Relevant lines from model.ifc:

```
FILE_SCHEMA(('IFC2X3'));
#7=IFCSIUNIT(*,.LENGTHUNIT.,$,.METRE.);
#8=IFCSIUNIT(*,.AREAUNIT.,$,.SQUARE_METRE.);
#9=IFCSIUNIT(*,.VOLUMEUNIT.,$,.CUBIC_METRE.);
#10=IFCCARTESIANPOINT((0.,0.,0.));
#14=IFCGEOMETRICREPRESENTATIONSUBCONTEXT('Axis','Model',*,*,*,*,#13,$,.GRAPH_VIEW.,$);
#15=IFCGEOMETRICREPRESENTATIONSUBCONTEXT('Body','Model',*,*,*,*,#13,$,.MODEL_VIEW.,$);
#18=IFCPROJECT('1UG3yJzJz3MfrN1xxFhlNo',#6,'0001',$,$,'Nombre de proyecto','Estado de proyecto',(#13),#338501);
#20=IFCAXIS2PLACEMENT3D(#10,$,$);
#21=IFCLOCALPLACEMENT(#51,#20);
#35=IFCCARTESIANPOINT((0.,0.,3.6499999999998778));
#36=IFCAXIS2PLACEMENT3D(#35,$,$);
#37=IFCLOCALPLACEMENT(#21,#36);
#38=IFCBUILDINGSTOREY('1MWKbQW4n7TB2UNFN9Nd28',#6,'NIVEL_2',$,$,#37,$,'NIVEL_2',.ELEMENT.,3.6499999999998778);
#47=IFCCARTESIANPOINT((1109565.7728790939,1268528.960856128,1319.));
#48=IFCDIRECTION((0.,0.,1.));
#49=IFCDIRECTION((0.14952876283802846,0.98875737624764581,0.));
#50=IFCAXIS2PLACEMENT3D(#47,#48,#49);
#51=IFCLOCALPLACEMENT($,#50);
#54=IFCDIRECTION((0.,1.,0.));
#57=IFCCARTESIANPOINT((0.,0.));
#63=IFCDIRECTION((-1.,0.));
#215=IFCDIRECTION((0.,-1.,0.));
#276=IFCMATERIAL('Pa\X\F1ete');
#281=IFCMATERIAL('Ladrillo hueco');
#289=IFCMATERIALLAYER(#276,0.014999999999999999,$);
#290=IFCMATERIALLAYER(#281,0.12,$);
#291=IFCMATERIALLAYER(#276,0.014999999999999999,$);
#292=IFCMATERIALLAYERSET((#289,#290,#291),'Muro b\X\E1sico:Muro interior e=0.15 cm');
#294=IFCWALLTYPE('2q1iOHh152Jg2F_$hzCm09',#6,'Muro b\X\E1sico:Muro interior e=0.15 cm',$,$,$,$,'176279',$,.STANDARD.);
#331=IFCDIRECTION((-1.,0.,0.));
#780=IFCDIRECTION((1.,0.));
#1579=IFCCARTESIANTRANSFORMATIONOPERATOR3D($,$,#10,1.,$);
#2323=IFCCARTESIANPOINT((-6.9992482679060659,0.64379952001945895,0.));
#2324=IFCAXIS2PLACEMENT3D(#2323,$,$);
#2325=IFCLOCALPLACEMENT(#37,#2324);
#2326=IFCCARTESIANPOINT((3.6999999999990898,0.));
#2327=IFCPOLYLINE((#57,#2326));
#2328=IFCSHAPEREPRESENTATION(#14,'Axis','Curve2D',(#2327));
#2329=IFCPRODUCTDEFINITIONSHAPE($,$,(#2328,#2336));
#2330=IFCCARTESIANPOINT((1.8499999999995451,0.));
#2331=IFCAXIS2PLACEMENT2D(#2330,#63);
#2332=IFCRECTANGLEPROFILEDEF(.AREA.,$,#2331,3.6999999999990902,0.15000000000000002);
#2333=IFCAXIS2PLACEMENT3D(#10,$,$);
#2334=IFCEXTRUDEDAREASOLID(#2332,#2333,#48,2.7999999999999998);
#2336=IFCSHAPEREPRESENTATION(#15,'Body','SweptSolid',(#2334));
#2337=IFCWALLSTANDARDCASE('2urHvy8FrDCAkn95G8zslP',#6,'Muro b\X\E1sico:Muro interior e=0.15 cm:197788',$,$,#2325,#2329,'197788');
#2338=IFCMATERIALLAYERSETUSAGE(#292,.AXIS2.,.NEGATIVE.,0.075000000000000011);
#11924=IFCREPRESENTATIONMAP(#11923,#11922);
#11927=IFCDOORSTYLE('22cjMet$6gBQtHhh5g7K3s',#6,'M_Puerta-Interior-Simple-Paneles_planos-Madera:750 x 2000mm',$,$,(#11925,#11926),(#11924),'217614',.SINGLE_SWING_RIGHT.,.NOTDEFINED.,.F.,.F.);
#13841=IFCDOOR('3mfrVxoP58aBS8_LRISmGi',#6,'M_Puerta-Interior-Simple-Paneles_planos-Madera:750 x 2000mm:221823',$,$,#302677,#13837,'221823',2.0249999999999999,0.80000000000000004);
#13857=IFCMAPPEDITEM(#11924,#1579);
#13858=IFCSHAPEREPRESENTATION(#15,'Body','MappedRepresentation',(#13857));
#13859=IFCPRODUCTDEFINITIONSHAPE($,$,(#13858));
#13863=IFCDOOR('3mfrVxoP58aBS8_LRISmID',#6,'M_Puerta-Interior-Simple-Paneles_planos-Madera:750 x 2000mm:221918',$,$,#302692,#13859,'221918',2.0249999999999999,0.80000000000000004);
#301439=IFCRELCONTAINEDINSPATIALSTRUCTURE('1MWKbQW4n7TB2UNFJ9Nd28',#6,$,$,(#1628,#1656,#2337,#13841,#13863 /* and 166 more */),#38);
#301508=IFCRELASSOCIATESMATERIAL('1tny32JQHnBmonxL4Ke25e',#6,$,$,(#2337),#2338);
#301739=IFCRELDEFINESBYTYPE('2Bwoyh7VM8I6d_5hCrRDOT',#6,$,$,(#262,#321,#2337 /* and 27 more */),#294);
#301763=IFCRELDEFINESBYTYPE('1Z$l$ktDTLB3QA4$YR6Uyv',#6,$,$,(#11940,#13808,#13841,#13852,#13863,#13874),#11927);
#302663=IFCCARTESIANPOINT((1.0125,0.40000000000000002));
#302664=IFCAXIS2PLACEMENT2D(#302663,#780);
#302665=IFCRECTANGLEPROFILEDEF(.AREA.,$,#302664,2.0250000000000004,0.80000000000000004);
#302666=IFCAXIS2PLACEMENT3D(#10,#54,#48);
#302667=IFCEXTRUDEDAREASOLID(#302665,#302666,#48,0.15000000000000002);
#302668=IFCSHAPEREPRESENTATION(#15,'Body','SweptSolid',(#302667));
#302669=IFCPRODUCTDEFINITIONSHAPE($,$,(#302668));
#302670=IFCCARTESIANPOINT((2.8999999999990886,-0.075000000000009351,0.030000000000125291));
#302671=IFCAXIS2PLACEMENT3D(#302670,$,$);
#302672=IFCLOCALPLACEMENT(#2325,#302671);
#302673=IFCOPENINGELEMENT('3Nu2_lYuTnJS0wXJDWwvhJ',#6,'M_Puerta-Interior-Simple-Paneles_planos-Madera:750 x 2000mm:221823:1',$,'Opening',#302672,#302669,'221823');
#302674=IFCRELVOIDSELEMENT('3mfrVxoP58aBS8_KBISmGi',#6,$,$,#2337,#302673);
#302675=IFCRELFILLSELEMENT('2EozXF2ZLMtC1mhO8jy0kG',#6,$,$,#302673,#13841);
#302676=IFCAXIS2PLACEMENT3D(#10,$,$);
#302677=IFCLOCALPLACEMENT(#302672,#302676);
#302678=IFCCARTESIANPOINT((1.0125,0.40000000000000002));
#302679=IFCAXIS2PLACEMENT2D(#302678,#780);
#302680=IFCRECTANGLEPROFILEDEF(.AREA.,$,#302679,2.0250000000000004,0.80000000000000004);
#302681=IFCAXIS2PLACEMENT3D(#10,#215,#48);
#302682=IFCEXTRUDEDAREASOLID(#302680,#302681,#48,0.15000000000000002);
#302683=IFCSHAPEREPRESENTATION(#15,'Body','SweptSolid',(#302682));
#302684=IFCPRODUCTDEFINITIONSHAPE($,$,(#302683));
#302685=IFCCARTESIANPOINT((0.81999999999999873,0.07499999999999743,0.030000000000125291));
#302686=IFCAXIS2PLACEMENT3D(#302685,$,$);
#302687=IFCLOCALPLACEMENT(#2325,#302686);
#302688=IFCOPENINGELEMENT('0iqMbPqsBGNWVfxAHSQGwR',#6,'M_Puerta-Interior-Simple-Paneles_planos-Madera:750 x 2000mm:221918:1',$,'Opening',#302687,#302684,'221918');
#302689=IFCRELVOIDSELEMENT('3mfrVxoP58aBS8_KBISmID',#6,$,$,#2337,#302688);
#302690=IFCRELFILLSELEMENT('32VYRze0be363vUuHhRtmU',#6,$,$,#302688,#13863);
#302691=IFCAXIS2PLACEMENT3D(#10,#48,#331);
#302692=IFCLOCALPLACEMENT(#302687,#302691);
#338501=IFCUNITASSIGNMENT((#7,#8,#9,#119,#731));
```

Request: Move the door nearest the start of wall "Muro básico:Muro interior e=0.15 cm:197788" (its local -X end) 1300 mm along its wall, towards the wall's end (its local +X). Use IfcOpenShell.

```python
import ifcopenshell
import ifcopenshell.api.geometry
import ifcopenshell.util.placement
import ifcopenshell.util.unit

model = ifcopenshell.open("model.ifc")
unit_scale = ifcopenshell.util.unit.calculate_unit_scale(model)

door = model.by_guid("3mfrVxoP58aBS8_LRISmID")
opening = door.FillsVoids[0].RelatingOpeningElement
wall = opening.VoidsElements[0].RelatingBuildingElement

wall_matrix = ifcopenshell.util.placement.get_local_placement(wall.ObjectPlacement)
shift = wall_matrix[:3, 0] * 1.3 / unit_scale
before = ifcopenshell.util.placement.get_local_placement(door.ObjectPlacement)[:3, 3].copy()

# The door is placed relative to its opening, so it follows when the opening moves.
matrix = ifcopenshell.util.placement.get_local_placement(opening.ObjectPlacement)
matrix[:3, 3] += shift
ifcopenshell.api.geometry.edit_object_placement(
    model, product=opening, matrix=matrix, is_si=False, should_transform_children=True
)

after = ifcopenshell.util.placement.get_local_placement(door.ObjectPlacement)[:3, 3]
print("door moved by", (after - before).round(3) + 0.0)

model.write("model-out.ifc")
```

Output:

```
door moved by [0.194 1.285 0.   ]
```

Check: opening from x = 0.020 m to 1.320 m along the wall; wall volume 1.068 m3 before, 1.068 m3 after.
